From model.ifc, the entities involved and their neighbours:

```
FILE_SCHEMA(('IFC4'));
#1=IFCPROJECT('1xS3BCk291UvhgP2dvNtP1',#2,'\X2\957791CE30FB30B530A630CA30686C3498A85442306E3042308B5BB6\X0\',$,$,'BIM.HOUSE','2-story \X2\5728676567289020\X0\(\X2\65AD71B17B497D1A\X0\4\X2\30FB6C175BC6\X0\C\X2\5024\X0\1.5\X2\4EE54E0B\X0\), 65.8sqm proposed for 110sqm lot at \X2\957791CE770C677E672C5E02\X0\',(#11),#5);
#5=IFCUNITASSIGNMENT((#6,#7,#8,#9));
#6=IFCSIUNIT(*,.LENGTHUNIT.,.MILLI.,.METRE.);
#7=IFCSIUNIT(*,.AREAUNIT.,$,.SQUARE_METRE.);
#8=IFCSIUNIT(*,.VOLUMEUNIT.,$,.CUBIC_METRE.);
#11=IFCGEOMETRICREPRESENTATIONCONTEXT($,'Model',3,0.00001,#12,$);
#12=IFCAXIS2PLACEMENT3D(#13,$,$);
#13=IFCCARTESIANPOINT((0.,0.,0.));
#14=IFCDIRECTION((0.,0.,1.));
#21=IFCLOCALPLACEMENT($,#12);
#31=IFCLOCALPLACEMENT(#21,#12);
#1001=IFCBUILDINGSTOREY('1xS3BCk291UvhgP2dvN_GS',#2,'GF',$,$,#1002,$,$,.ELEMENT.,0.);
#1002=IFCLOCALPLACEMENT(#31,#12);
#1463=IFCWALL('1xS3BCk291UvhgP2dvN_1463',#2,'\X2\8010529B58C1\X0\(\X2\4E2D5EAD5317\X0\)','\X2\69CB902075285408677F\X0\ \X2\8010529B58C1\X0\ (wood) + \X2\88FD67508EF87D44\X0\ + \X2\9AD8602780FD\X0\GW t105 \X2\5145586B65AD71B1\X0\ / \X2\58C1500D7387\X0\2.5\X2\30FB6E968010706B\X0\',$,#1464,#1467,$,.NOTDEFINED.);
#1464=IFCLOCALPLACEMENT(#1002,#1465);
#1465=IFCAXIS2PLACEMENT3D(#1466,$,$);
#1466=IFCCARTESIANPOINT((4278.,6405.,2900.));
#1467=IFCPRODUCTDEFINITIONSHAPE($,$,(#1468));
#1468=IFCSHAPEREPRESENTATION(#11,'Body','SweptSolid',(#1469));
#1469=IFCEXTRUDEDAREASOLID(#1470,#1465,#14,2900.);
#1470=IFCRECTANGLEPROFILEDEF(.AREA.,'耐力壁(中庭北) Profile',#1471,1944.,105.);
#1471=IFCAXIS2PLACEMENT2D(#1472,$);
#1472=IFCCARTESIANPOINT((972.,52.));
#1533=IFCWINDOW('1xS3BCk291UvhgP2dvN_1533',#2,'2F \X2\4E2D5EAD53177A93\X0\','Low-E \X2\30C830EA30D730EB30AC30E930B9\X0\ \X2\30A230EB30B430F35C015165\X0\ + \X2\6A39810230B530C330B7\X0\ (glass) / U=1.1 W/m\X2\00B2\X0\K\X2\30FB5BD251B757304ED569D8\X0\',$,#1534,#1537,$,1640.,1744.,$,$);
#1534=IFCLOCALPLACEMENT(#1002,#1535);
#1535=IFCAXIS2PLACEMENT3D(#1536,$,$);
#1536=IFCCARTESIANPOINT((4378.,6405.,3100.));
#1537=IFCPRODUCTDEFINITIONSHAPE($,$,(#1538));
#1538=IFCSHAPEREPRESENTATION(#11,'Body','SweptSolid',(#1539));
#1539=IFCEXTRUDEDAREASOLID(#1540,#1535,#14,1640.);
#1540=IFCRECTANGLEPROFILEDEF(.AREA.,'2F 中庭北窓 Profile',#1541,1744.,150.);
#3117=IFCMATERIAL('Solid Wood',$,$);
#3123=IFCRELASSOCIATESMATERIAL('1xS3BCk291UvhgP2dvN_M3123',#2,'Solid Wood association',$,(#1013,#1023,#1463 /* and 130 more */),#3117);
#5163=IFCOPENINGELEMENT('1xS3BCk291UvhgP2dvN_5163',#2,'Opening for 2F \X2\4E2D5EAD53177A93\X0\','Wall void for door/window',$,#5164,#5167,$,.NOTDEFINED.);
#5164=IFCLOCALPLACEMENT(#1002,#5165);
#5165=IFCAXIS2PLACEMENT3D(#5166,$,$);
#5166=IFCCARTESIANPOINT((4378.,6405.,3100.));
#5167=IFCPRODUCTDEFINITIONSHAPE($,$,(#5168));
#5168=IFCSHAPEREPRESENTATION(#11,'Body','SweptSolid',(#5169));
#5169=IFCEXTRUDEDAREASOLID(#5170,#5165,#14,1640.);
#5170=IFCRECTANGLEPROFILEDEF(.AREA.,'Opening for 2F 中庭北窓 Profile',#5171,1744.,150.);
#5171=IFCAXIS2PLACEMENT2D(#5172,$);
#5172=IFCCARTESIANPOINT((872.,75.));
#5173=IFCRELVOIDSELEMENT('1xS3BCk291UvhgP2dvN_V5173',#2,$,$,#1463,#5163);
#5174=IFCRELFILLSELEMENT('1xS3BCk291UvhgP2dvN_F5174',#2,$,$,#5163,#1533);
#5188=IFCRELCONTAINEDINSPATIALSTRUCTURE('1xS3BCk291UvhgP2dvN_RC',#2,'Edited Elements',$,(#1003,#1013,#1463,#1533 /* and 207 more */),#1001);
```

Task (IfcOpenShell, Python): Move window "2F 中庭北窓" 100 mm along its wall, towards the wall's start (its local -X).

```python
import ifcopenshell
import ifcopenshell.api.geometry
import ifcopenshell.util.placement
import ifcopenshell.util.unit

model = ifcopenshell.open("model.ifc")
unit_scale = ifcopenshell.util.unit.calculate_unit_scale(model)

window = model.by_guid("1xS3BCk291UvhgP2dvN_1533")
opening = window.FillsVoids[0].RelatingOpeningElement
wall = opening.VoidsElements[0].RelatingBuildingElement

wall_matrix = ifcopenshell.util.placement.get_local_placement(wall.ObjectPlacement)
shift = wall_matrix[:3, 0] * -0.1 / unit_scale
before = ifcopenshell.util.placement.get_local_placement(window.ObjectPlacement)[:3, 3].copy()

# The window is not placed relative to its opening, so move both.
for product in (opening, window):
    matrix = ifcopenshell.util.placement.get_local_placement(product.ObjectPlacement)
    matrix[:3, 3] += shift
    ifcopenshell.api.geometry.edit_object_placement(model, product=product, matrix=matrix, is_si=False)

after = ifcopenshell.util.placement.get_local_placement(window.ObjectPlacement)[:3, 3]
print("window moved by", (after - before).round(3) + 0.0)

model.write("model_updated.ifc")
```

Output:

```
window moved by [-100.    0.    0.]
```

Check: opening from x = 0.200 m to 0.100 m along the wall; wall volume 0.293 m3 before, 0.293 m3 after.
